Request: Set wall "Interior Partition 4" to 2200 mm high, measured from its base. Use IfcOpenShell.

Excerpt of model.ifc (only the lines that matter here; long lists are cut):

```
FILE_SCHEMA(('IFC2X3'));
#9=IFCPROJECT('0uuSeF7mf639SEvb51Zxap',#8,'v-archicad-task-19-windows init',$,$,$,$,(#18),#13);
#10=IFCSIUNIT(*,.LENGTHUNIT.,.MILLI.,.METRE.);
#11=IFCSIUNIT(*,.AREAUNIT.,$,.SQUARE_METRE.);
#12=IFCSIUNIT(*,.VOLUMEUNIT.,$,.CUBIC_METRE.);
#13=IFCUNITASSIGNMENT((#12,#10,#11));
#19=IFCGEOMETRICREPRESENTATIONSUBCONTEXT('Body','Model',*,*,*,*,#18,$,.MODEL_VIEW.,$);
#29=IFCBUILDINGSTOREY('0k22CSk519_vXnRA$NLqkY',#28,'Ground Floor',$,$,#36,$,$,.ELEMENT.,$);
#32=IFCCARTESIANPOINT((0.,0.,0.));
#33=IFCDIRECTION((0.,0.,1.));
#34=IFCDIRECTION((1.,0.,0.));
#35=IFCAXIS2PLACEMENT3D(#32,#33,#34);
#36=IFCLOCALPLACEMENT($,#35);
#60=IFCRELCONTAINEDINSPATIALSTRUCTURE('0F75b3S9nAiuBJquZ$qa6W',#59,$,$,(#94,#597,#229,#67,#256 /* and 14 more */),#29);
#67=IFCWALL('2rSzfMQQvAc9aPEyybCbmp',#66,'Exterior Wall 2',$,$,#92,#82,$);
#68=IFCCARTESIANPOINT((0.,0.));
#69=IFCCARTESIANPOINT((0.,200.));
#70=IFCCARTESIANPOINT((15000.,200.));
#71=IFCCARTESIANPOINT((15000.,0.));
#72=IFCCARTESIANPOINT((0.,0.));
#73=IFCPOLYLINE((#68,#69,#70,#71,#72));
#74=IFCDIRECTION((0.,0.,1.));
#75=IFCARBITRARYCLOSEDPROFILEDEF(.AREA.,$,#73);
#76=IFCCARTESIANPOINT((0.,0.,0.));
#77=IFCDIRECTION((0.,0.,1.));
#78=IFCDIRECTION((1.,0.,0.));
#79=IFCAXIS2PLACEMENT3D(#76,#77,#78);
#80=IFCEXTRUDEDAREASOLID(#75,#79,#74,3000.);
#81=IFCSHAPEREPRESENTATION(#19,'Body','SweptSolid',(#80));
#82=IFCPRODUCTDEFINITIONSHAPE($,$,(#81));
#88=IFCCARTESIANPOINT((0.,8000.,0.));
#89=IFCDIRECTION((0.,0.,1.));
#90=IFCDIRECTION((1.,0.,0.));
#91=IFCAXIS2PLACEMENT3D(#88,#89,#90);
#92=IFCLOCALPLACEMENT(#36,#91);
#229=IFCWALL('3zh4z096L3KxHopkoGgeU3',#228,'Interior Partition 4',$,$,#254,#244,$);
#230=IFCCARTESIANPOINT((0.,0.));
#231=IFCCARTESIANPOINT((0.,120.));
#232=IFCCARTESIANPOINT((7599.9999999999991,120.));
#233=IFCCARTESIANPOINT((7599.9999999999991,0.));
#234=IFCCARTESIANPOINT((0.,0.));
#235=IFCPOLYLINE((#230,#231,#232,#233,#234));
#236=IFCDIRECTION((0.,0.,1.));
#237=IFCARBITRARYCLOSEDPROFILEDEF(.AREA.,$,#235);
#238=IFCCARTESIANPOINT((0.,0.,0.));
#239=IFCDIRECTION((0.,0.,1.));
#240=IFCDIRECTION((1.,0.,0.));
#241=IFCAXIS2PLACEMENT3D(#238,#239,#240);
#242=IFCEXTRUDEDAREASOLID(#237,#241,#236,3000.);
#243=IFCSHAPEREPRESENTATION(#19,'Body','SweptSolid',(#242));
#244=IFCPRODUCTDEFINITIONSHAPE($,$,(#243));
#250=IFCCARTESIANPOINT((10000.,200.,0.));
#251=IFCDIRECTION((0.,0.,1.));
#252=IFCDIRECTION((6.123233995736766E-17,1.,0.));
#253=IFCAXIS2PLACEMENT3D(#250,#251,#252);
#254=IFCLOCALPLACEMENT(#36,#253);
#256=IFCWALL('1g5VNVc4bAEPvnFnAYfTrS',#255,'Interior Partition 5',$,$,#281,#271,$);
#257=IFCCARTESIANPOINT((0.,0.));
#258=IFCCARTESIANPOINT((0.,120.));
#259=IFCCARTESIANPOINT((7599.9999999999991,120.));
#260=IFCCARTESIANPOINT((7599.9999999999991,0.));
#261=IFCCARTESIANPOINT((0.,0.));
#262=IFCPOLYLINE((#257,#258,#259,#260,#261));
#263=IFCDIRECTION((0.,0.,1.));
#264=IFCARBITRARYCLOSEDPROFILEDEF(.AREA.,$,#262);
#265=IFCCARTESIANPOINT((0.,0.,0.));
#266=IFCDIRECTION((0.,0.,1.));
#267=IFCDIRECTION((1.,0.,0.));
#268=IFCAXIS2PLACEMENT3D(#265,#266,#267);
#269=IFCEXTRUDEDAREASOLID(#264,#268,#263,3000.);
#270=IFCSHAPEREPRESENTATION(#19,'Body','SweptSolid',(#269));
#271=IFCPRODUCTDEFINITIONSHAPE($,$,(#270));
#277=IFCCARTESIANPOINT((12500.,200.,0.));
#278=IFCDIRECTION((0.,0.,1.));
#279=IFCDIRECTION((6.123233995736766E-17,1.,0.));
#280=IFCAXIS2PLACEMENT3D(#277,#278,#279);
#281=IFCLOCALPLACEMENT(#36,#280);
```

```python
import ifcopenshell
import ifcopenshell.geom
import ifcopenshell.util.representation
import ifcopenshell.util.shape
import ifcopenshell.util.unit

model = ifcopenshell.open("model.ifc")
unit_scale = ifcopenshell.util.unit.calculate_unit_scale(model)
settings = ifcopenshell.geom.settings()


def volume(element):
    """Net volume in cubic metres, openings subtracted."""
    shape = ifcopenshell.geom.create_shape(settings, element)
    return ifcopenshell.util.shape.get_volume(shape.geometry)


wall = model.by_guid("3zh4z096L3KxHopkoGgeU3")
before = volume(wall)

body = ifcopenshell.util.representation.get_representation(wall, "Model", "Body")
solid = body.Items[0]
old_height = solid.Depth
solid.Depth = 2.2 / unit_scale
after = volume(wall)

print(f"height {old_height:g} -> {solid.Depth:g}, volume {before:.3f} -> {after:.3f} m3")

model.write("model-out.ifc")
```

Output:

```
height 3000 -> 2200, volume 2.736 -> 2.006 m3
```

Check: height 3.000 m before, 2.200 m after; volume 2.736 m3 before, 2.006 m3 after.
